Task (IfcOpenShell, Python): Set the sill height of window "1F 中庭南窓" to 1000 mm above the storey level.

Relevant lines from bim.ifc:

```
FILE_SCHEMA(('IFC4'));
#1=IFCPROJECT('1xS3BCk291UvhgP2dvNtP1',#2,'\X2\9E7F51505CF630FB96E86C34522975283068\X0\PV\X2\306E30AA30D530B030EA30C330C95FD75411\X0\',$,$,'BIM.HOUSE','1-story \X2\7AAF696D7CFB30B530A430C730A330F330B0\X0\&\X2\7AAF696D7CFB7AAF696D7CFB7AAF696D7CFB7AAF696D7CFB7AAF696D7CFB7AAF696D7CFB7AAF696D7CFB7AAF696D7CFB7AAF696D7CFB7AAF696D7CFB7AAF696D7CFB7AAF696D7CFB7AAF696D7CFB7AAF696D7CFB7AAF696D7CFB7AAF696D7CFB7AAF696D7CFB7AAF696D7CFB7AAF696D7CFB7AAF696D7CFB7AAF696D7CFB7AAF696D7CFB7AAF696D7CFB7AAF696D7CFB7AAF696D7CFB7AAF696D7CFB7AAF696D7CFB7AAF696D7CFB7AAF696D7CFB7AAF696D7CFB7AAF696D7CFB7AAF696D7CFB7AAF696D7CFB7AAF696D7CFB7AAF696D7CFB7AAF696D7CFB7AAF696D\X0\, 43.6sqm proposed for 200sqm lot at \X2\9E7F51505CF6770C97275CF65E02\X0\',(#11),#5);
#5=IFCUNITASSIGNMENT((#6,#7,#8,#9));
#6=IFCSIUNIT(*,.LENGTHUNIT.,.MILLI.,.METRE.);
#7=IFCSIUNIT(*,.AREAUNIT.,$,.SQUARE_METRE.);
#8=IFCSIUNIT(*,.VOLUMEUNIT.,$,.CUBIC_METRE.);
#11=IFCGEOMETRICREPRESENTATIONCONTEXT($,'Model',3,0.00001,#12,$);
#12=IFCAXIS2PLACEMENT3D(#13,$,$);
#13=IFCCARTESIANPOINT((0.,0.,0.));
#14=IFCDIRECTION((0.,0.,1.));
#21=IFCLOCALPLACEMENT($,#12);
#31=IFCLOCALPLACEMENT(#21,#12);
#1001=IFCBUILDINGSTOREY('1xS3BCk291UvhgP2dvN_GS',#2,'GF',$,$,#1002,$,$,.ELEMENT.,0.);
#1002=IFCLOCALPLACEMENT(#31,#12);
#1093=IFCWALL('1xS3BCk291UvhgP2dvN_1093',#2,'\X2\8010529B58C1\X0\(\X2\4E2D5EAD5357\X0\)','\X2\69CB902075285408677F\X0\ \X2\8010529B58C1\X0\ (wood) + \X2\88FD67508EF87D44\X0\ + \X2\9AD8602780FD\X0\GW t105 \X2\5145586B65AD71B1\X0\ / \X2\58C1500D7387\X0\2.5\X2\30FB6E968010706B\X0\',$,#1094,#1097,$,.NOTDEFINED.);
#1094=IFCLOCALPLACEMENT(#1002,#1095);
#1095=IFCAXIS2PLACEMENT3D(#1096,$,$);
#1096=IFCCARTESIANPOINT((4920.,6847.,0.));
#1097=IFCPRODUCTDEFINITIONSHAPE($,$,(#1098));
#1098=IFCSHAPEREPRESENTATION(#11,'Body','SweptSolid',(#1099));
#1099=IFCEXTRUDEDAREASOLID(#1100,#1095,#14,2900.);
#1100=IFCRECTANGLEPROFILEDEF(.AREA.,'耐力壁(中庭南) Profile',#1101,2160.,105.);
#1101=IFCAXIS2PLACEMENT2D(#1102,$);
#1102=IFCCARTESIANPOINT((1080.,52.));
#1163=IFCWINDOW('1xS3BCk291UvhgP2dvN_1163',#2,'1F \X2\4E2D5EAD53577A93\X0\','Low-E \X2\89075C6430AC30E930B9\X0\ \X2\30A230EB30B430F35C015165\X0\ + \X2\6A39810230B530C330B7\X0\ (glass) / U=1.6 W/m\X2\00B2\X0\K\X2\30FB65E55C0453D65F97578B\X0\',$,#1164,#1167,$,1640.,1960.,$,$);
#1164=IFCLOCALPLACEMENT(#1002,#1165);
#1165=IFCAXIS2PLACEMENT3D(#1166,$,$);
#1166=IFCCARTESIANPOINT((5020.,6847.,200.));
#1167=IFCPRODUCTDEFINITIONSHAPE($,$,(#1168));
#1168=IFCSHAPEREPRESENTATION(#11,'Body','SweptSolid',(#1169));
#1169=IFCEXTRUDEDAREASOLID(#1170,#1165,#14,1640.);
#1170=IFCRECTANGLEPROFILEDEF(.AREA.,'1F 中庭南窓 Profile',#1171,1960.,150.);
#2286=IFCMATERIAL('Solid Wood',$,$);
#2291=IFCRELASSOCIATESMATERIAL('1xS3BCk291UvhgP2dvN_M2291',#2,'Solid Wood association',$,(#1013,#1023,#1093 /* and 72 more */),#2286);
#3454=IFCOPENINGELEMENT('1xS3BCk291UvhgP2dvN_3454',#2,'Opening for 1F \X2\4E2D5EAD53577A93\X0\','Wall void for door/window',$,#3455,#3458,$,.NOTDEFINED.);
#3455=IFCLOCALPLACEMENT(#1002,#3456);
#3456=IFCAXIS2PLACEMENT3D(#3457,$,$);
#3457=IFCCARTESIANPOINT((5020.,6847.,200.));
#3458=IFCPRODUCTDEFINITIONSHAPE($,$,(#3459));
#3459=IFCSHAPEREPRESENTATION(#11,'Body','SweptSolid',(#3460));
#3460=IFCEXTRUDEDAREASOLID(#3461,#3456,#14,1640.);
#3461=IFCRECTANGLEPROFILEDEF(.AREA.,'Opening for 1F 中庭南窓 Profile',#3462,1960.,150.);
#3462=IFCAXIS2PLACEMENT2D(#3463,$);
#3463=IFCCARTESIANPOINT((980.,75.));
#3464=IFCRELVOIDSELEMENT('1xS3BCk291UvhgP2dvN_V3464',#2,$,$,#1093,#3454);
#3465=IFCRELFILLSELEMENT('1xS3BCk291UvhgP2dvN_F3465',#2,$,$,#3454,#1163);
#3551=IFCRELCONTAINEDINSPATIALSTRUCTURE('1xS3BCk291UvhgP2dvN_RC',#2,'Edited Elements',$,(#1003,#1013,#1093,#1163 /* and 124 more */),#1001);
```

```python
import numpy as np
import ifcopenshell
import ifcopenshell.api.geometry
import ifcopenshell.geom
import ifcopenshell.util.element
import ifcopenshell.util.placement
import ifcopenshell.util.shape
import ifcopenshell.util.unit

model = ifcopenshell.open("bim.ifc")
unit_scale = ifcopenshell.util.unit.calculate_unit_scale(model)

window = model.by_guid("1xS3BCk291UvhgP2dvN_1163")
opening = window.FillsVoids[0].RelatingOpeningElement
storey = ifcopenshell.util.element.get_container(window, ifc_class="IfcBuildingStorey")
level = ifcopenshell.util.placement.get_local_placement(storey.ObjectPlacement)[2, 3]

# The opening's origin need not be at the sill, so measure its lowest point.
shape = ifcopenshell.geom.create_shape(ifcopenshell.geom.settings(), opening)
bottom = ifcopenshell.util.shape.get_shape_bottom_elevation(shape, shape.geometry) / unit_scale
dz = level + 1 / unit_scale - bottom

shift = np.array([0.0, 0.0, dz])
# The window is not placed relative to its opening, so move both.
for product in (opening, window):
    matrix = ifcopenshell.util.placement.get_local_placement(product.ObjectPlacement)
    matrix[:3, 3] += shift
    ifcopenshell.api.geometry.edit_object_placement(model, product=product, matrix=matrix, is_si=False)

print(f"moved by {dz * unit_scale:+.3f} m")

model.write("bim-out.ifc")
```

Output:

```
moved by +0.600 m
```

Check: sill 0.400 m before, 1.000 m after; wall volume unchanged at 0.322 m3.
